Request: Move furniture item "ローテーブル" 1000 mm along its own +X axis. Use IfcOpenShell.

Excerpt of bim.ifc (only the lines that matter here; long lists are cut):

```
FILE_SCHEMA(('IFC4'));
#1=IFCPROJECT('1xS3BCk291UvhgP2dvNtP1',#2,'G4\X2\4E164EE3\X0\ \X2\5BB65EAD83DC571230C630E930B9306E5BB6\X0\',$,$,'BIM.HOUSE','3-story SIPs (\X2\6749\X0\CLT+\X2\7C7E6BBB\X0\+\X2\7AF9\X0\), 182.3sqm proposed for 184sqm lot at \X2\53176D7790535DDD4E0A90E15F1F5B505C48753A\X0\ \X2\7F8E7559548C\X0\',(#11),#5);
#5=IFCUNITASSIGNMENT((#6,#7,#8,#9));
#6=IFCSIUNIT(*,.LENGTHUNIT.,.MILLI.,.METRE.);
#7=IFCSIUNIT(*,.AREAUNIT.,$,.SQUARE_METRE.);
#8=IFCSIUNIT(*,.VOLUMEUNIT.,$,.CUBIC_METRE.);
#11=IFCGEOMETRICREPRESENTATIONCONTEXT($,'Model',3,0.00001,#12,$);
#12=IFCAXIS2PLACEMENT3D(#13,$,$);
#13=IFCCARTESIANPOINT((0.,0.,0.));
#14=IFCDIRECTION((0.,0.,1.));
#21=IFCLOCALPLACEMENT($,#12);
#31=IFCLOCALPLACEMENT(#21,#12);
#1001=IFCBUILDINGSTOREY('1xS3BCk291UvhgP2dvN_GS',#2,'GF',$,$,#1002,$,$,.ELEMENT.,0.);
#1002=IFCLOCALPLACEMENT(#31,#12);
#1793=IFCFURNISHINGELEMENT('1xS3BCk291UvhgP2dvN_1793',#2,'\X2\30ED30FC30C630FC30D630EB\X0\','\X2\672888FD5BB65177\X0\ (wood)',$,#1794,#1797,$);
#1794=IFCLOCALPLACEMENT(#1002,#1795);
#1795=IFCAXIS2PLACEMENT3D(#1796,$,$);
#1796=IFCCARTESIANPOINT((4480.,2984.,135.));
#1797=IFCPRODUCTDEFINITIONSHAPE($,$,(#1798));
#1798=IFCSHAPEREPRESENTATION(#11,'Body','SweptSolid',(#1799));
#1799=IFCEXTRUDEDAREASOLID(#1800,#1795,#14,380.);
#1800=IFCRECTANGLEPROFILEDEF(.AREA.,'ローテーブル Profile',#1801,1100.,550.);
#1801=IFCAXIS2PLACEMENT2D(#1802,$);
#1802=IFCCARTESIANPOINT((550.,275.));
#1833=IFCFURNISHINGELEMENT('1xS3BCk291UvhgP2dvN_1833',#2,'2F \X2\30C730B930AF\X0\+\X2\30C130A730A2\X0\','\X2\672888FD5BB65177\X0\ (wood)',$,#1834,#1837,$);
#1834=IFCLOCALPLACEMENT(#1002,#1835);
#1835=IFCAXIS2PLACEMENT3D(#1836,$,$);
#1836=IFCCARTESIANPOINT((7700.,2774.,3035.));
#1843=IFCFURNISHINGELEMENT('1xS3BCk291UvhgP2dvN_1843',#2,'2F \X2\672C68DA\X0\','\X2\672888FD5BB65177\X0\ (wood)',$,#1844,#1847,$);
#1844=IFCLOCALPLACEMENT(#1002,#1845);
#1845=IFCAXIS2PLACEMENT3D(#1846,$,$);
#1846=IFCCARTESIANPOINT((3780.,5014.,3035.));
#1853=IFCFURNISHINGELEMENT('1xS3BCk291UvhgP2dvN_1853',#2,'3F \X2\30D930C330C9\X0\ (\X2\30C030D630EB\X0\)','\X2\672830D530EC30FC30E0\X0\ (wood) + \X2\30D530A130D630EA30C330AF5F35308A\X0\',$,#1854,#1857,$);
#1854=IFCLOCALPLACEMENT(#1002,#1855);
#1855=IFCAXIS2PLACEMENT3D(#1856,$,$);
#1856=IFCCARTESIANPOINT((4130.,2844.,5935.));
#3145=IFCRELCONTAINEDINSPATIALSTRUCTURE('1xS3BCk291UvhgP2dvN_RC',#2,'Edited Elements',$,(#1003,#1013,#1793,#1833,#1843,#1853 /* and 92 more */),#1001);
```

```python
import ifcopenshell
import ifcopenshell.api.geometry
import ifcopenshell.util.placement

model = ifcopenshell.open("bim.ifc")

item = model.by_guid("1xS3BCk291UvhgP2dvN_1793")
matrix = ifcopenshell.util.placement.get_local_placement(item.ObjectPlacement)
matrix[:3, 3] += matrix[:3, 0] * 1000.0
ifcopenshell.api.geometry.edit_object_placement(model, product=item, matrix=matrix, is_si=False)

print(ifcopenshell.util.placement.get_local_placement(item.ObjectPlacement).round(3) + 0.0)

model.write("bim-out.ifc")
```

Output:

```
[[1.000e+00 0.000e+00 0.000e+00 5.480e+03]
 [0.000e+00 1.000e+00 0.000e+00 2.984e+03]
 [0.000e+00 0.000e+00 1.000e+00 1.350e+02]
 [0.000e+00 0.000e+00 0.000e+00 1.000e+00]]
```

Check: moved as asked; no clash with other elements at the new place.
